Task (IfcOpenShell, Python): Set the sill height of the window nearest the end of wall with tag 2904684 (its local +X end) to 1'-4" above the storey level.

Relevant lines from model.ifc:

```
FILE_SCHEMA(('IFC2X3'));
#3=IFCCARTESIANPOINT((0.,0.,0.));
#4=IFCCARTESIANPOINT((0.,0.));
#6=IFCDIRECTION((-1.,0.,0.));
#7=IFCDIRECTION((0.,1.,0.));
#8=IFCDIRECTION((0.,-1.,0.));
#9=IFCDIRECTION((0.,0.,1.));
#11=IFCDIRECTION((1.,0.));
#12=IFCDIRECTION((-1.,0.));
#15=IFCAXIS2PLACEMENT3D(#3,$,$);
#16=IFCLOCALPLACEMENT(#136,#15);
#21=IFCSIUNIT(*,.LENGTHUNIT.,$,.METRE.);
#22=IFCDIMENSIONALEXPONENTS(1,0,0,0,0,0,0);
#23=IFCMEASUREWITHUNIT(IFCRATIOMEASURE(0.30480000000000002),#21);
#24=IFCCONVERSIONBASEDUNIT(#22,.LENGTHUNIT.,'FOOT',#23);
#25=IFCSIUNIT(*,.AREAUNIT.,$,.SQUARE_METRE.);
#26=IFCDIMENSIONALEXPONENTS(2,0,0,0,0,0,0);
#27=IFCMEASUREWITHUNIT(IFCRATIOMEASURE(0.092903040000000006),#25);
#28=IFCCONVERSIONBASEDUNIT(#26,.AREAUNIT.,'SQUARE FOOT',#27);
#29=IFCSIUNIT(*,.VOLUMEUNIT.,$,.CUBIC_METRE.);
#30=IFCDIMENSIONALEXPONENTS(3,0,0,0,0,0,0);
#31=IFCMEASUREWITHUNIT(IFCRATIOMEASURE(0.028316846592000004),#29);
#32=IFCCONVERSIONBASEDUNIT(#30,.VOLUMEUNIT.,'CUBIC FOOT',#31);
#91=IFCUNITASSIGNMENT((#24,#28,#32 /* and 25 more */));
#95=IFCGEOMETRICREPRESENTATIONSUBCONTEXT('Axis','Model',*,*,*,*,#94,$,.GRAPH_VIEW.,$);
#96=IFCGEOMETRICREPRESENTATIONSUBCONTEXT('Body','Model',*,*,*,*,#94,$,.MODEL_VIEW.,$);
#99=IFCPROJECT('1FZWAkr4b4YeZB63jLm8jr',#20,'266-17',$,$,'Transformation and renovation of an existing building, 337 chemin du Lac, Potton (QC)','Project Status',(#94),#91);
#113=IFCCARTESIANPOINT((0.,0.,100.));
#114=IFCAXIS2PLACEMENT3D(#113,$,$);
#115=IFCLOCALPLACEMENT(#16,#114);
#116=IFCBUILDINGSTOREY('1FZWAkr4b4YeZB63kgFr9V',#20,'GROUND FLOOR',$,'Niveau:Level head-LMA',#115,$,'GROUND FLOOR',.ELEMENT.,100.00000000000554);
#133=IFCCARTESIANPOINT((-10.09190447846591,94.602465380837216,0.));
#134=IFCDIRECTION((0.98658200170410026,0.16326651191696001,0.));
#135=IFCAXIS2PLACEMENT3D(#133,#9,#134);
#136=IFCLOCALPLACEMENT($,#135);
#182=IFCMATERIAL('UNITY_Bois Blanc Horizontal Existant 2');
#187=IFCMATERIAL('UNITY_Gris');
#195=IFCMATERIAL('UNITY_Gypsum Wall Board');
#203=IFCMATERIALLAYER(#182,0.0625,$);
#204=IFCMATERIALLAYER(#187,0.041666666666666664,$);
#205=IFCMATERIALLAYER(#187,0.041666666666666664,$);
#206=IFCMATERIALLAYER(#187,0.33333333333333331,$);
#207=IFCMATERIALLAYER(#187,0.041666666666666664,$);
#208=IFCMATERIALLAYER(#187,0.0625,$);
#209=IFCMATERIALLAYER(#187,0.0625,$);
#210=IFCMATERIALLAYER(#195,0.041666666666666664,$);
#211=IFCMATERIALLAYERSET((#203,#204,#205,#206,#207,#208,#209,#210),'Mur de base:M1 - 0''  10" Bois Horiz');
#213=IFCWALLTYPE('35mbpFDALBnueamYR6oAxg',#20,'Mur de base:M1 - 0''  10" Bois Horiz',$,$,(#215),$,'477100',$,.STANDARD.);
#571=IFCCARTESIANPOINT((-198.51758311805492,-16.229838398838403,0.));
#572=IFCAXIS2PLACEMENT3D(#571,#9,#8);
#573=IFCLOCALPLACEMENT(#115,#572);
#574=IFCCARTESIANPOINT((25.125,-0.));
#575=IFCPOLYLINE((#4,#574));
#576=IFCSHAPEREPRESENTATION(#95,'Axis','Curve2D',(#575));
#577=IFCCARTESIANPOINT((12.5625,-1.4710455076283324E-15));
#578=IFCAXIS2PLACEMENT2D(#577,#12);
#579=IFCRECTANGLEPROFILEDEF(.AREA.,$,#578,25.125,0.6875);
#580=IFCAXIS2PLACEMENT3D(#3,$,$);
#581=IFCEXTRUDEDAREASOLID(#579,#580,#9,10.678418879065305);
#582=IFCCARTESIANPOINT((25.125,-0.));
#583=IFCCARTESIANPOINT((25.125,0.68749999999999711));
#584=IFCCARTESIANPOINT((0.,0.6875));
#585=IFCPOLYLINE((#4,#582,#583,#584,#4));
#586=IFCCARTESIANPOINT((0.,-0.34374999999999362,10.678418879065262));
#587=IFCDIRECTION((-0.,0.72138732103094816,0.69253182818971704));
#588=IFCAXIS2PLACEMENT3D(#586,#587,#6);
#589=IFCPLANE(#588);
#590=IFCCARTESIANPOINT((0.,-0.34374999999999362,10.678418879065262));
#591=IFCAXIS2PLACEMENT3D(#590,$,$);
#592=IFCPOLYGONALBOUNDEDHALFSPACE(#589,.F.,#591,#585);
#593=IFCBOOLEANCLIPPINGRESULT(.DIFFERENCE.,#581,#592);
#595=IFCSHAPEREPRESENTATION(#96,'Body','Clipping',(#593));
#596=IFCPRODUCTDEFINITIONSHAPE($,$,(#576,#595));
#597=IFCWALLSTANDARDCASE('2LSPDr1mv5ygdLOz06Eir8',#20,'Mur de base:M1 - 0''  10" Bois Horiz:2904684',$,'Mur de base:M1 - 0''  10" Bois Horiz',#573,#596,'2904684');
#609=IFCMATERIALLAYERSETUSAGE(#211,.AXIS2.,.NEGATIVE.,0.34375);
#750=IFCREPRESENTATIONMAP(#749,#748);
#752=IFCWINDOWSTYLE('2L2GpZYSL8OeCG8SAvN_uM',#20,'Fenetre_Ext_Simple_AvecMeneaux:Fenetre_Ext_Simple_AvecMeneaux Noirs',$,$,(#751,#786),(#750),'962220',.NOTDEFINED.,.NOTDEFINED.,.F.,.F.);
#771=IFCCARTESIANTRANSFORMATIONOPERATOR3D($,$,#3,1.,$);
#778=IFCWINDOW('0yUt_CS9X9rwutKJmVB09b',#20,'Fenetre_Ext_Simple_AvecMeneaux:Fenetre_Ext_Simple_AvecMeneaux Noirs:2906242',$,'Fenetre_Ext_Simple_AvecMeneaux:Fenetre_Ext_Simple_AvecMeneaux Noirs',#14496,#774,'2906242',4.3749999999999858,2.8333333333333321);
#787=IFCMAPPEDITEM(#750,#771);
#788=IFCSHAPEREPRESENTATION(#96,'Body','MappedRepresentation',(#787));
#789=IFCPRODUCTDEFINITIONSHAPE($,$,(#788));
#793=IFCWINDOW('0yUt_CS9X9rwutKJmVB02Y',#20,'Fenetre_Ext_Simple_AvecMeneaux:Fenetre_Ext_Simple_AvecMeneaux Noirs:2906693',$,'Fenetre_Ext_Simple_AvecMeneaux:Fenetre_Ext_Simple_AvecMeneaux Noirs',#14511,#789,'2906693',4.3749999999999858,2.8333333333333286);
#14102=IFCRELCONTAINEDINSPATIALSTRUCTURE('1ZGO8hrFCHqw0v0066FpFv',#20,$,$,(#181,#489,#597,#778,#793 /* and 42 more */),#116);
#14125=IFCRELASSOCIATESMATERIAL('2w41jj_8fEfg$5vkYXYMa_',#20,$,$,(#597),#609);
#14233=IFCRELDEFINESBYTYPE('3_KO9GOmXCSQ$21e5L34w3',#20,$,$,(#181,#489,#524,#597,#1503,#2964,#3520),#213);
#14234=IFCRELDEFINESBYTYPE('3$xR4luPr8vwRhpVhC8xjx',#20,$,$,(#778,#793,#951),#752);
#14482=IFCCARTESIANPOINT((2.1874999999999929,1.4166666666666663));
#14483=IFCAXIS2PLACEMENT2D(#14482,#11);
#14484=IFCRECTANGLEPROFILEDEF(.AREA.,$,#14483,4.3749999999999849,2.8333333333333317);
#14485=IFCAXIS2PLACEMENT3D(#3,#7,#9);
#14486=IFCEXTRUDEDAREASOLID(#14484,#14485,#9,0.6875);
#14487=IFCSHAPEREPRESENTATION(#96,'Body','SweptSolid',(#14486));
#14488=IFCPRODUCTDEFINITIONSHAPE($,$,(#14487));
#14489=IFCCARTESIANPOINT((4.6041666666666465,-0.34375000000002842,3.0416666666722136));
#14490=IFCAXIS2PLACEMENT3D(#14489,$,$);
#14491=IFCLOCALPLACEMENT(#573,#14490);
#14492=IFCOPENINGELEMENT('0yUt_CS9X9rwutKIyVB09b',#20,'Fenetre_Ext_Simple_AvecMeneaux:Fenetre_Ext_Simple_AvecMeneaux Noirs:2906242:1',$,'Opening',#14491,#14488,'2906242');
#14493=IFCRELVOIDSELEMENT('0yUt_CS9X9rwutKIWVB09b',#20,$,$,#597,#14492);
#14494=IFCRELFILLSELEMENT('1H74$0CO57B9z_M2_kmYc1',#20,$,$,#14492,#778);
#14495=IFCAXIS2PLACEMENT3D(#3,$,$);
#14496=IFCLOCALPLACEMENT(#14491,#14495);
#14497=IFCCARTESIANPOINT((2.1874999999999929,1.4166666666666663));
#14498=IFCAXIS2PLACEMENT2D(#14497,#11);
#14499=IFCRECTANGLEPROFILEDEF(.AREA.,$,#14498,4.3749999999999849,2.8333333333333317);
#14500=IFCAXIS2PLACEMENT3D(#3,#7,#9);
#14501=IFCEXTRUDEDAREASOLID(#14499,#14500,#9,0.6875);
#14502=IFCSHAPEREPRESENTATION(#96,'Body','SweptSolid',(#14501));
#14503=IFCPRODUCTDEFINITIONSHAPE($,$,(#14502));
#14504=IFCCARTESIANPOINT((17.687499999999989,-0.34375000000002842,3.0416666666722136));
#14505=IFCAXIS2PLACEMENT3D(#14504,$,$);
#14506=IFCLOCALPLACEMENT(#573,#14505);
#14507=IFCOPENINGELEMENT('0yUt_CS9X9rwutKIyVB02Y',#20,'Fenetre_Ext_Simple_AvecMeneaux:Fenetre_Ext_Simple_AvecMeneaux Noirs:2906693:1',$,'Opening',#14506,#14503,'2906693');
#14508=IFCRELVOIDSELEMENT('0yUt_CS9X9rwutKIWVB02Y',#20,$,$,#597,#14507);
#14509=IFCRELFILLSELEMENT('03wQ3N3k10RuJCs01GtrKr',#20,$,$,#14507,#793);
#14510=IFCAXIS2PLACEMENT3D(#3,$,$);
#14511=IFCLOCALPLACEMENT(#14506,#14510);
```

```python
import numpy as np
import ifcopenshell
import ifcopenshell.api.geometry
import ifcopenshell.geom
import ifcopenshell.util.element
import ifcopenshell.util.placement
import ifcopenshell.util.shape
import ifcopenshell.util.unit

model = ifcopenshell.open("model.ifc")
unit_scale = ifcopenshell.util.unit.calculate_unit_scale(model)

window = model.by_guid("0yUt_CS9X9rwutKJmVB02Y")
opening = window.FillsVoids[0].RelatingOpeningElement
storey = ifcopenshell.util.element.get_container(window, ifc_class="IfcBuildingStorey")
level = ifcopenshell.util.placement.get_local_placement(storey.ObjectPlacement)[2, 3]

# The opening's origin need not be at the sill, so measure its lowest point.
shape = ifcopenshell.geom.create_shape(ifcopenshell.geom.settings(), opening)
bottom = ifcopenshell.util.shape.get_shape_bottom_elevation(shape, shape.geometry) / unit_scale
dz = level + 16 * 0.0254 / unit_scale - bottom

shift = np.array([0.0, 0.0, dz])
# The window is placed relative to its opening, so it follows when the opening moves.
matrix = ifcopenshell.util.placement.get_local_placement(opening.ObjectPlacement)
matrix[:3, 3] += shift
ifcopenshell.api.geometry.edit_object_placement(
    model, product=opening, matrix=matrix, is_si=False, should_transform_children=True
)

print(f"moved by {dz * unit_scale:+.3f} m")

model.write("model_edited.ifc")
```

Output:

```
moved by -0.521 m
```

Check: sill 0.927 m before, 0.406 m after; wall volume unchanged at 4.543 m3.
